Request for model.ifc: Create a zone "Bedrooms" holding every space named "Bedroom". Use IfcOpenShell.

First a look at what the model holds.

```python
import ifcopenshell

model = ifcopenshell.open("model.ifc")
print(model.schema)
seen = {}
for space in model.by_type("IfcSpace"):
    seen[space.LongName] = seen.get(space.LongName, 0) + 1
for name, count in sorted(seen.items(), key=str):
    print(count, "x", name)
print("zones:", [z.Name for z in model.by_type("IfcZone")][:20])
```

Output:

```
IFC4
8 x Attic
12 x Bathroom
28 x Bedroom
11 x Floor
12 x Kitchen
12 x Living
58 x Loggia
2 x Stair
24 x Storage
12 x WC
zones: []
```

```python
import ifcopenshell
import ifcopenshell.api.group
import ifcopenshell.api.root

model = ifcopenshell.open("model.ifc")

names = {"Bedroom"}
spaces = [s for s in model.by_type("IfcSpace") if s.LongName in names]

zone = ifcopenshell.api.root.create_entity(model, ifc_class="IfcZone", name="Bedrooms")
ifcopenshell.api.group.assign_group(model, products=spaces, group=zone)
print(len(spaces), "spaces in", zone.Name)

model.write("model_rev.ifc")
```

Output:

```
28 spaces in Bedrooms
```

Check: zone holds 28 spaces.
